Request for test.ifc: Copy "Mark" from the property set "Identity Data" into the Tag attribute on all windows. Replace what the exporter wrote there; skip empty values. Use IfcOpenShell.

First a look at what the model holds.

```python
import ifcopenshell
import ifcopenshell.util.element

model = ifcopenshell.open("test.ifc")
print(model.schema)
windows = model.by_type("IfcWindow")
print(len(windows), "windows")
for e in windows[:8]:
    source = ifcopenshell.util.element.get_pset(e, "Identity Data", "Mark")
    target = e.Tag
    print(e.id(), repr(source), repr(target), sep=" | ")
```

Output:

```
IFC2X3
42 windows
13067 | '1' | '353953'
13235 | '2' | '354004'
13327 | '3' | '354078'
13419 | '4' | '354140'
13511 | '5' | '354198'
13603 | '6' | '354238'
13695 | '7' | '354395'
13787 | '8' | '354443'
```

```python
import ifcopenshell
import ifcopenshell.util.element

model = ifcopenshell.open("test.ifc")

count = 0
for e in model.by_type("IfcWindow"):
    value = ifcopenshell.util.element.get_pset(e, "Identity Data", "Mark")
    current = e.Tag
    if not value or not value.strip() or current == value:
        continue
    e.Tag = value
    count += 1

print(count, "windows updated")

model.write("test_rev.ifc")
```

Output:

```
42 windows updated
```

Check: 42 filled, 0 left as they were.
